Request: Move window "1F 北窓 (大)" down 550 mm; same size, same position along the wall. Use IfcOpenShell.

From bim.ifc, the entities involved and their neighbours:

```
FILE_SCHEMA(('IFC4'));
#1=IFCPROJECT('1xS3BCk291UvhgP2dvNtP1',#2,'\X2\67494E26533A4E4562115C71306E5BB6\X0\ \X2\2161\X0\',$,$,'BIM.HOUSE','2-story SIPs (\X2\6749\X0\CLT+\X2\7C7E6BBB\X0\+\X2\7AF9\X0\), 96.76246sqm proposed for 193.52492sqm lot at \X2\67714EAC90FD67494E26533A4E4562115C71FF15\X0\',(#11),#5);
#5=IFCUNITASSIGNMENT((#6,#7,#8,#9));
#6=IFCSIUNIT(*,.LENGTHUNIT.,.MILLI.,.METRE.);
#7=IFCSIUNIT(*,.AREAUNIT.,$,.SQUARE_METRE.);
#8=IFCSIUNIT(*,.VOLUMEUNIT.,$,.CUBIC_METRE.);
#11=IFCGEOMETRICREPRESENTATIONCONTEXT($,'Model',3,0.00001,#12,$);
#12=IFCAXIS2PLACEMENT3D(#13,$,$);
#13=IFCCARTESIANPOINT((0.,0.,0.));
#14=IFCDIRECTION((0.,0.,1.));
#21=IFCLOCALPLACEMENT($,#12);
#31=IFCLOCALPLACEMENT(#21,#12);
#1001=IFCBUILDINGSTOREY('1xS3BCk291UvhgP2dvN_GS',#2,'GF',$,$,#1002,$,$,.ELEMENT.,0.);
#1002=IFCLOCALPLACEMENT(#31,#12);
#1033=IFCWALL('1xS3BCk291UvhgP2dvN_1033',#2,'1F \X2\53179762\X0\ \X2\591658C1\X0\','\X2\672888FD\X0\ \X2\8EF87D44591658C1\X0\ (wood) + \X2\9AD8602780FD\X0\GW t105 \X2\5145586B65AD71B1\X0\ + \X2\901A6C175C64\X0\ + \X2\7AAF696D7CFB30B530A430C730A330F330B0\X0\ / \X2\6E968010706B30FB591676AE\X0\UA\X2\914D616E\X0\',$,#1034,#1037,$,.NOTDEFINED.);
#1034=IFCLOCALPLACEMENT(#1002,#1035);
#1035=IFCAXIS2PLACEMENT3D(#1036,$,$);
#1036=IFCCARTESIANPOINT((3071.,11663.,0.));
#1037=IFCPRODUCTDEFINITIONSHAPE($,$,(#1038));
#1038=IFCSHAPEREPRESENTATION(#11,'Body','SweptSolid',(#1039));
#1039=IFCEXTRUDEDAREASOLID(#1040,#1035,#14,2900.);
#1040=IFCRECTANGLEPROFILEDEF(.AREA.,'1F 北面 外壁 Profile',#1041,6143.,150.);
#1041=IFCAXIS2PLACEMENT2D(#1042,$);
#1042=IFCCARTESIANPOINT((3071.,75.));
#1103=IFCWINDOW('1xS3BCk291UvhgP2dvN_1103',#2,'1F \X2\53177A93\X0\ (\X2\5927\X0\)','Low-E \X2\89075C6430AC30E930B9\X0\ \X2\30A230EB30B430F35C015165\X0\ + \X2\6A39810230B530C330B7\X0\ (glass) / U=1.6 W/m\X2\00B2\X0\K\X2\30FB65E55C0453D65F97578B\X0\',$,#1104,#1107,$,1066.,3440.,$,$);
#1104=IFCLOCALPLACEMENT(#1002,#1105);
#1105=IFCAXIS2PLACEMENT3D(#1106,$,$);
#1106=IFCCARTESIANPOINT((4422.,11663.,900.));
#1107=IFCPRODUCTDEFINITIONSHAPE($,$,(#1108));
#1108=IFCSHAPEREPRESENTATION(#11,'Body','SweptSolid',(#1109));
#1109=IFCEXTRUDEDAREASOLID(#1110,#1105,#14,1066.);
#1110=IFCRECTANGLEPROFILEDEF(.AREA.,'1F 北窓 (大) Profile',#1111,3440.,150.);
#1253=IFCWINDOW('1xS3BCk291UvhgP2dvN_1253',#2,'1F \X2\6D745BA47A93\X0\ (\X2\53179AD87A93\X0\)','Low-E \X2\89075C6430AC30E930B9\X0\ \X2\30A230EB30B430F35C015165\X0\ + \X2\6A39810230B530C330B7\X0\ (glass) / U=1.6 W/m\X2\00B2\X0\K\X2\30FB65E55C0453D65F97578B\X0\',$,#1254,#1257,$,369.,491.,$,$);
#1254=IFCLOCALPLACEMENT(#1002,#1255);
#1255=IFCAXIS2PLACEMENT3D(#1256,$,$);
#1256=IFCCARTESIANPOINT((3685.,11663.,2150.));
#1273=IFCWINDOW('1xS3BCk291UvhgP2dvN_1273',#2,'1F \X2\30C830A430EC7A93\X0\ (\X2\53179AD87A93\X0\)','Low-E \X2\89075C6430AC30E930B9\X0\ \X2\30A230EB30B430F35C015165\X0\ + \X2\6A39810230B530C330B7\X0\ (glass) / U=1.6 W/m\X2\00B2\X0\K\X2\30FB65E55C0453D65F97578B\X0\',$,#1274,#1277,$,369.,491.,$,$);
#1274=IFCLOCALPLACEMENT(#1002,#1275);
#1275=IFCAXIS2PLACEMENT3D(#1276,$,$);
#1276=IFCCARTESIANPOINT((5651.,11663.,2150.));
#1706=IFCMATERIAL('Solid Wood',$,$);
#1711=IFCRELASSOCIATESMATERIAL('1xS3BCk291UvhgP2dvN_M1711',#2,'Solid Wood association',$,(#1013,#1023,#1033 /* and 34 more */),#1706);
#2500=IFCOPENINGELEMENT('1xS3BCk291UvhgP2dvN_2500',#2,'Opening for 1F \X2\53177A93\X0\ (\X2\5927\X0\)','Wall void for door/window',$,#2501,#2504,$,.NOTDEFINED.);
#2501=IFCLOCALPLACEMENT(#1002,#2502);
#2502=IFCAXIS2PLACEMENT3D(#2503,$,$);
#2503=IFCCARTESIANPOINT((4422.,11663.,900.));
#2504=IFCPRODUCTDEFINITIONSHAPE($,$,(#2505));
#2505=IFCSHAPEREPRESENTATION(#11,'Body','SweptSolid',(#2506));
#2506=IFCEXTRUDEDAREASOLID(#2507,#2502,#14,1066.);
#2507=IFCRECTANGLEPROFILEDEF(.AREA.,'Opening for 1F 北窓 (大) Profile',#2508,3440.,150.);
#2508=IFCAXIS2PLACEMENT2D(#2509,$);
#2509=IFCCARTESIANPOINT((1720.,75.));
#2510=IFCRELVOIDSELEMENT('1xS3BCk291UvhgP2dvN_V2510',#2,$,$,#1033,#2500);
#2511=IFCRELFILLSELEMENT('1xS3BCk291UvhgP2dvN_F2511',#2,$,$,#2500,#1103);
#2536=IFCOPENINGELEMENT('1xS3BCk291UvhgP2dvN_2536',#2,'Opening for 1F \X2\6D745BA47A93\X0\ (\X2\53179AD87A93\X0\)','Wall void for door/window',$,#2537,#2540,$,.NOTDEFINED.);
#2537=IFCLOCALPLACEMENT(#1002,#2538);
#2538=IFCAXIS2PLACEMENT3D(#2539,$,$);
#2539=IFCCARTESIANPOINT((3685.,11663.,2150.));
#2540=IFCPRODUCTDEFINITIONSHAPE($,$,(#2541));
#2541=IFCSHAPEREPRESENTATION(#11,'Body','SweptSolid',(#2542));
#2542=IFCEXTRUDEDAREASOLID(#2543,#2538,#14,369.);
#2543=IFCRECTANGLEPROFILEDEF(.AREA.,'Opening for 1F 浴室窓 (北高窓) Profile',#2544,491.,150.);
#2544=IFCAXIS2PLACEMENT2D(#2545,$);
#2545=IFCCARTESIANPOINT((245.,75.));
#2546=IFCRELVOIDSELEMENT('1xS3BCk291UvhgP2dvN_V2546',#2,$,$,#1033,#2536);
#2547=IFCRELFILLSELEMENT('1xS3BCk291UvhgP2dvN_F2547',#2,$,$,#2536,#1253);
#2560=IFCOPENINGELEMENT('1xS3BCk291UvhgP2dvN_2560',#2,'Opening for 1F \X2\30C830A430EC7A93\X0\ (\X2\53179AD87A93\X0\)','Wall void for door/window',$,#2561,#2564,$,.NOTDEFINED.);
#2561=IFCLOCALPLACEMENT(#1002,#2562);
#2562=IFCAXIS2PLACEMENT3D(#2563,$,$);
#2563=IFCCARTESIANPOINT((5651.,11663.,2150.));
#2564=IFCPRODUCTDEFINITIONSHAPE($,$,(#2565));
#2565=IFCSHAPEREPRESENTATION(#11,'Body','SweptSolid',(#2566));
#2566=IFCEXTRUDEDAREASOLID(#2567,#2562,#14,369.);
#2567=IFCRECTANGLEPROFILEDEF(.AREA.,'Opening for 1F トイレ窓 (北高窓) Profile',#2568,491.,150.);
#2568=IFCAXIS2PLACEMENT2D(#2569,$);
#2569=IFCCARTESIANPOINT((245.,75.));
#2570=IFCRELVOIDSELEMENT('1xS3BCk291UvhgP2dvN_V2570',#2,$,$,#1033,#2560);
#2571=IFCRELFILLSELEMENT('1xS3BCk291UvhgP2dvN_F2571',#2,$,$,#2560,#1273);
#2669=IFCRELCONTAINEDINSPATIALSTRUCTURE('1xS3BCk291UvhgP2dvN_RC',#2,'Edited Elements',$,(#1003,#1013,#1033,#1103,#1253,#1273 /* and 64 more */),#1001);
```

```python
import numpy as np
import ifcopenshell
import ifcopenshell.api.geometry
import ifcopenshell.util.placement
import ifcopenshell.util.unit

model = ifcopenshell.open("bim.ifc")
unit_scale = ifcopenshell.util.unit.calculate_unit_scale(model)

window = model.by_guid("1xS3BCk291UvhgP2dvN_1103")
opening = window.FillsVoids[0].RelatingOpeningElement
dz = -0.55 / unit_scale

shift = np.array([0.0, 0.0, dz])
# The window is not placed relative to its opening, so move both.
for product in (opening, window):
    matrix = ifcopenshell.util.placement.get_local_placement(product.ObjectPlacement)
    matrix[:3, 3] += shift
    ifcopenshell.api.geometry.edit_object_placement(model, product=product, matrix=matrix, is_si=False)

print(f"moved by {dz * unit_scale:+.3f} m")

model.write("bim_v2.ifc")
```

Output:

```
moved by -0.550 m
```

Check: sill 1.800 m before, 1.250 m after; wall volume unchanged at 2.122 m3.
